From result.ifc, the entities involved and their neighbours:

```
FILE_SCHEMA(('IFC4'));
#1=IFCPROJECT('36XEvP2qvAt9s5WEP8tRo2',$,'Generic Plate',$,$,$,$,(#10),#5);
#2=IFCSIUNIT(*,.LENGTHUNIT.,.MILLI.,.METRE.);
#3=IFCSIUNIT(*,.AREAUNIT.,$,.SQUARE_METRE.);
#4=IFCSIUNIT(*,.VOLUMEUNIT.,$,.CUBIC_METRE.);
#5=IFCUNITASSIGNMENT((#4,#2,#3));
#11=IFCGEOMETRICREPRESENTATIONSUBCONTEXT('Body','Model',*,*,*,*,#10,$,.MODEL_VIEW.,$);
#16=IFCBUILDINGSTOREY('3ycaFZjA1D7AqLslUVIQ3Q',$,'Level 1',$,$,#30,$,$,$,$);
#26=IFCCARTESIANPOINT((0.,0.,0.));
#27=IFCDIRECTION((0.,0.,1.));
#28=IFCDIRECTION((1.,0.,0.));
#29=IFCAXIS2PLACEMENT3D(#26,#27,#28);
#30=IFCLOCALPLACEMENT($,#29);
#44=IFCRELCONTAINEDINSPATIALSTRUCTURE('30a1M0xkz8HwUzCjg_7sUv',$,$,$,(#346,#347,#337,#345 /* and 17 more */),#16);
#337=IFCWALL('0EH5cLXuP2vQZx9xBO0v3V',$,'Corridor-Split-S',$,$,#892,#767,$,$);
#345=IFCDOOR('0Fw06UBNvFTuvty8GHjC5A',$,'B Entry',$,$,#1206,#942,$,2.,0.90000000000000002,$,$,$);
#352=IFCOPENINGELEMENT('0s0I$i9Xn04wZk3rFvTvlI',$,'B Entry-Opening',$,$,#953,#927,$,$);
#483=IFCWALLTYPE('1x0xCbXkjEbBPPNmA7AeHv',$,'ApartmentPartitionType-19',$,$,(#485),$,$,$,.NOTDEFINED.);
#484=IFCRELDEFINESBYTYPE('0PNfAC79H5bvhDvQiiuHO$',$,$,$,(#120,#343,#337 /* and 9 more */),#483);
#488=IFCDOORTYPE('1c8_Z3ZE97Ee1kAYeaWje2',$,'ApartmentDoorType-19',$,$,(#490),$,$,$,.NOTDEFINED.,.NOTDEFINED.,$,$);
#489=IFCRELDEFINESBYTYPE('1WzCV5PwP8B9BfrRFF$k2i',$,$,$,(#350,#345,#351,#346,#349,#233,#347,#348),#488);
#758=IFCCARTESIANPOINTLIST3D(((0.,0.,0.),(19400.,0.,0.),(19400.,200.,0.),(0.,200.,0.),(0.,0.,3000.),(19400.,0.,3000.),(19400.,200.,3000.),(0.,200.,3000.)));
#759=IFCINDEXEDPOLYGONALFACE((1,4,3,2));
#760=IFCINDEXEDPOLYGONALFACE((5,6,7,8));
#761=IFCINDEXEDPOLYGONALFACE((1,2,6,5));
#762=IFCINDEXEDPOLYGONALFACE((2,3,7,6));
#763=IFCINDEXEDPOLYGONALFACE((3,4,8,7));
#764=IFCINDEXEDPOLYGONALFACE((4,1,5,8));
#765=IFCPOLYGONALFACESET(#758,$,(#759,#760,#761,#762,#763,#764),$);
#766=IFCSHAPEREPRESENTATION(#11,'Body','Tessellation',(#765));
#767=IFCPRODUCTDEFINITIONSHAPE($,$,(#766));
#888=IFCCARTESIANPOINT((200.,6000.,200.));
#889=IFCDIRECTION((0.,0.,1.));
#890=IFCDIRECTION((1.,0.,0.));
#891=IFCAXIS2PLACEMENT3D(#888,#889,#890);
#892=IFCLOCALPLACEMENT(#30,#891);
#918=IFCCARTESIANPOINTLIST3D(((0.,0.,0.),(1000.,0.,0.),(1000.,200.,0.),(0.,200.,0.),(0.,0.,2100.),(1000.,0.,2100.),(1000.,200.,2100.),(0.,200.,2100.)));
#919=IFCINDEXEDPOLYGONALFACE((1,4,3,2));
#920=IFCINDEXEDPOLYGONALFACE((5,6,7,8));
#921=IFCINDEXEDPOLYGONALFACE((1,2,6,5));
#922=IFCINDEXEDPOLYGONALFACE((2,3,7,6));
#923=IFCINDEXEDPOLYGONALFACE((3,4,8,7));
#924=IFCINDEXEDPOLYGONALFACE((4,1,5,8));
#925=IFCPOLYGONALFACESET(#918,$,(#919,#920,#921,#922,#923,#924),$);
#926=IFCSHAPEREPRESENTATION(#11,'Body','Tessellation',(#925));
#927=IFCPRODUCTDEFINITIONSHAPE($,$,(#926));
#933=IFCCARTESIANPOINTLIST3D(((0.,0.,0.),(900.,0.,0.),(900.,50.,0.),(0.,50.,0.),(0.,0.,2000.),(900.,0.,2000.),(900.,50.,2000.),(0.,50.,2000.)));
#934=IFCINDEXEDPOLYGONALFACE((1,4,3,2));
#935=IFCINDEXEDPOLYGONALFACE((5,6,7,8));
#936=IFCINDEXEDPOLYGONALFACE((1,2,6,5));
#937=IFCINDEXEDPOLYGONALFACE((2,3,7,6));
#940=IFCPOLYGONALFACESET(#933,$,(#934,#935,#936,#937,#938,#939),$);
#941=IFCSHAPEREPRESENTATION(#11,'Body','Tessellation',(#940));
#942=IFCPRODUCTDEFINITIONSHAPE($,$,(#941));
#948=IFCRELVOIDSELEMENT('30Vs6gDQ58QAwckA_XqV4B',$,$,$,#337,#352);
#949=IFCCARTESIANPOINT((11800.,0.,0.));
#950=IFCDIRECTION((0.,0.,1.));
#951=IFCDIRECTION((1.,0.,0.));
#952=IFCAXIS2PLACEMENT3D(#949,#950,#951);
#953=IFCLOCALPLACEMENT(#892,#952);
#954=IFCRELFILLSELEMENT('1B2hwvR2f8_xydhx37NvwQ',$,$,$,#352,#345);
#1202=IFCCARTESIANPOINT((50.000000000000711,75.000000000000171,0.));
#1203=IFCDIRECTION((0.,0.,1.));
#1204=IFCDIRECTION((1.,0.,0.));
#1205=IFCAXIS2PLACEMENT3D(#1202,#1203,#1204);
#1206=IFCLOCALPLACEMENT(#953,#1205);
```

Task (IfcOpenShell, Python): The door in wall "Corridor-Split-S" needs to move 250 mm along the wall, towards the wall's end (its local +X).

```python
import ifcopenshell
import ifcopenshell.api.geometry
import ifcopenshell.util.placement

model = ifcopenshell.open("result.ifc")

door = model.by_guid("0Fw06UBNvFTuvty8GHjC5A")
opening = door.FillsVoids[0].RelatingOpeningElement
wall = opening.VoidsElements[0].RelatingBuildingElement

wall_matrix = ifcopenshell.util.placement.get_local_placement(wall.ObjectPlacement)
shift = wall_matrix[:3, 0] * 250.0
before = ifcopenshell.util.placement.get_local_placement(door.ObjectPlacement)[:3, 3].copy()

# The door is placed relative to its opening, so it follows when the opening moves.
matrix = ifcopenshell.util.placement.get_local_placement(opening.ObjectPlacement)
matrix[:3, 3] += shift
ifcopenshell.api.geometry.edit_object_placement(
    model, product=opening, matrix=matrix, is_si=False, should_transform_children=True
)

after = ifcopenshell.util.placement.get_local_placement(door.ObjectPlacement)[:3, 3]
print("door moved by", (after - before).round(3) + 0.0)

model.write("result_v2.ifc")
```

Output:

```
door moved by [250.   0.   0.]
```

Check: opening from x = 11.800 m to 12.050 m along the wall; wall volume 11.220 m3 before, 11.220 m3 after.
